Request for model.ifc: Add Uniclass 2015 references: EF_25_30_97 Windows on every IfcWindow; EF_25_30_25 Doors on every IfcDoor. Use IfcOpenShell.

First a look at what the model holds.

```python
import ifcopenshell

model = ifcopenshell.open("model.ifc")
print(model.schema)
print("classifications:", [c.Name for c in model.by_type("IfcClassification")])
for ifc_class in ("IfcDoor", "IfcRoof", "IfcStair", "IfcWall", "IfcWindow"):
    print(ifc_class, len(model.by_type(ifc_class)))
```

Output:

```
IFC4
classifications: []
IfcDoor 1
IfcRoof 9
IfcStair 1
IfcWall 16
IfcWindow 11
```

```python
import ifcopenshell
import ifcopenshell.api.classification

model = ifcopenshell.open("model.ifc")

system = ifcopenshell.api.classification.add_classification(model, classification="Uniclass 2015")

codes = {
    "IfcWindow": ("EF_25_30_97", "Windows"),
    "IfcDoor": ("EF_25_30_25", "Doors"),
}
for ifc_class, (code, name) in codes.items():
    products = model.by_type(ifc_class)
    ifcopenshell.api.classification.add_reference(
        model, products=products, classification=system, identification=code, name=name
    )
    print(code, len(products))

model.write("model_updated.ifc")
```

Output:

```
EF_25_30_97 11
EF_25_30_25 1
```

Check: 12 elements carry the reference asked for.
